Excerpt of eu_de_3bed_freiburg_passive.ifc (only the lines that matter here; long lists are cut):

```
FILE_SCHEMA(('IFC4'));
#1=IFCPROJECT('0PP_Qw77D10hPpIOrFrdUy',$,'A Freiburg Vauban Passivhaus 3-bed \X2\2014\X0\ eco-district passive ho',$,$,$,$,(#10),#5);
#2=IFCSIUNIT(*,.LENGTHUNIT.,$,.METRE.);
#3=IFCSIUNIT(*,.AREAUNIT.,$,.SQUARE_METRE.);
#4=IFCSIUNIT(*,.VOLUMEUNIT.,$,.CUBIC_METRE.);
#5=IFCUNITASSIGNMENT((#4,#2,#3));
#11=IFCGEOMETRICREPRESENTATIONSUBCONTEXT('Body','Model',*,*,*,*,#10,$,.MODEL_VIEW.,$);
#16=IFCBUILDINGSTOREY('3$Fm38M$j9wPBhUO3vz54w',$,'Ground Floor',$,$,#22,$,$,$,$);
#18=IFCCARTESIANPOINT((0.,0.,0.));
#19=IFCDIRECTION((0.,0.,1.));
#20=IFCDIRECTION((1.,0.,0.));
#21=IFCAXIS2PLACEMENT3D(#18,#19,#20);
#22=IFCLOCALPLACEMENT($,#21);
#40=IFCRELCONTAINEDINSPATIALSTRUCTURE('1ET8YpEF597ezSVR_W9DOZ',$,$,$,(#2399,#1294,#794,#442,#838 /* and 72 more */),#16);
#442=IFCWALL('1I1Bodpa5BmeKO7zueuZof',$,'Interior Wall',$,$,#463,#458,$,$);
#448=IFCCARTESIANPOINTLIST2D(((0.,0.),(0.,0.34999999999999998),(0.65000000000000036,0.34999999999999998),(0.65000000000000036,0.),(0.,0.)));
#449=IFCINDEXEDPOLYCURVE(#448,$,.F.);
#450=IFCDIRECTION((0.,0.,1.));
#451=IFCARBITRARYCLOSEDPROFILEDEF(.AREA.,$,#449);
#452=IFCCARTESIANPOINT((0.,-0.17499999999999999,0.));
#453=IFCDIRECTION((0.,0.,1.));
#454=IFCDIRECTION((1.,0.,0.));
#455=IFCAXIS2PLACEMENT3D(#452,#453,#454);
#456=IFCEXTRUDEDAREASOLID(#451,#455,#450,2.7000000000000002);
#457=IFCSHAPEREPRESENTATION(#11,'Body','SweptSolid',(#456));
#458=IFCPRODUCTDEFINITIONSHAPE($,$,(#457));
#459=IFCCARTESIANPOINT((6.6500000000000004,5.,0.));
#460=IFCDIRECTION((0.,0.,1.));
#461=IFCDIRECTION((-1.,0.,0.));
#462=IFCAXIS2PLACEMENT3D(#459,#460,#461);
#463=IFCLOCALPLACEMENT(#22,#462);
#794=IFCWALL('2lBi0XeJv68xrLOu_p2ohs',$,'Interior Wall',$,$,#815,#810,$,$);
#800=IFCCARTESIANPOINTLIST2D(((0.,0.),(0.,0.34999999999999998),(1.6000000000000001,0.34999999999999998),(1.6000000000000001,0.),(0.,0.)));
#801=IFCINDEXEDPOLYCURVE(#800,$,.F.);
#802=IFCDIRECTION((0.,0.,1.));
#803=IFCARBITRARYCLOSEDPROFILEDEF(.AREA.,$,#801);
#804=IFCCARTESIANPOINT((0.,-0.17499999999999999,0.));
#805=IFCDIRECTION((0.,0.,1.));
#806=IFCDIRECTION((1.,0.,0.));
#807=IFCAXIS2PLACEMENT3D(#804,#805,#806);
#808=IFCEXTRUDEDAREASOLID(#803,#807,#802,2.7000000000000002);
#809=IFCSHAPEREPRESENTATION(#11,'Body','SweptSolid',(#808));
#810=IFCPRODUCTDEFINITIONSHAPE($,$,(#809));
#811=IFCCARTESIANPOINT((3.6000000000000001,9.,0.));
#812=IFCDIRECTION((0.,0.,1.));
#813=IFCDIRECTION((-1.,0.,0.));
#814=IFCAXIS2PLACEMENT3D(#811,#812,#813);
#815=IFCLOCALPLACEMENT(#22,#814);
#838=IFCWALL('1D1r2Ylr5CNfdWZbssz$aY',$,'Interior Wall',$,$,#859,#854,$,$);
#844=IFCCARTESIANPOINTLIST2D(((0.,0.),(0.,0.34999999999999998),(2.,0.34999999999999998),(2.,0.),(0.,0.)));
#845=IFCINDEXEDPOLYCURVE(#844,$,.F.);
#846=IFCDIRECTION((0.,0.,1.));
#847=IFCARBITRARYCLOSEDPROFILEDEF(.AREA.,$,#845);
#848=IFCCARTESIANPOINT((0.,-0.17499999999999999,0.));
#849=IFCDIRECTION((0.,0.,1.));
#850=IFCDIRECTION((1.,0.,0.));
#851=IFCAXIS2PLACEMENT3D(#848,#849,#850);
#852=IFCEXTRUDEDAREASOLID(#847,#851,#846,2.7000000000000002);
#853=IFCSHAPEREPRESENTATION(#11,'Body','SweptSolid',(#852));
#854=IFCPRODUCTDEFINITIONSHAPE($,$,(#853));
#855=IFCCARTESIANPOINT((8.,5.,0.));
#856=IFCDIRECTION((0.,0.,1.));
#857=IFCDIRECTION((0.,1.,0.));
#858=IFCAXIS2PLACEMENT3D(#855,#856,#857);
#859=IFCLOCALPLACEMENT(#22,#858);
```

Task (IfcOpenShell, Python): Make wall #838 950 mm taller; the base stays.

```python
import ifcopenshell
import ifcopenshell.geom
import ifcopenshell.util.representation
import ifcopenshell.util.shape

model = ifcopenshell.open("eu_de_3bed_freiburg_passive.ifc")
settings = ifcopenshell.geom.settings()


def volume(element):
    """Net volume in cubic metres, openings subtracted."""
    shape = ifcopenshell.geom.create_shape(settings, element)
    return ifcopenshell.util.shape.get_volume(shape.geometry)


wall = model.by_id(838)
before = volume(wall)

body = ifcopenshell.util.representation.get_representation(wall, "Model", "Body")
solid = body.Items[0]
old_height = solid.Depth
solid.Depth += 0.95
after = volume(wall)

print(f"height {old_height:g} -> {solid.Depth:g}, volume {before:.3f} -> {after:.3f} m3")

model.write("eu_de_3bed_freiburg_passive-out.ifc")
```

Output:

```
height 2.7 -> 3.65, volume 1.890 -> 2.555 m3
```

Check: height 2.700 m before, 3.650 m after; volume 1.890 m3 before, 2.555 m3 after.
